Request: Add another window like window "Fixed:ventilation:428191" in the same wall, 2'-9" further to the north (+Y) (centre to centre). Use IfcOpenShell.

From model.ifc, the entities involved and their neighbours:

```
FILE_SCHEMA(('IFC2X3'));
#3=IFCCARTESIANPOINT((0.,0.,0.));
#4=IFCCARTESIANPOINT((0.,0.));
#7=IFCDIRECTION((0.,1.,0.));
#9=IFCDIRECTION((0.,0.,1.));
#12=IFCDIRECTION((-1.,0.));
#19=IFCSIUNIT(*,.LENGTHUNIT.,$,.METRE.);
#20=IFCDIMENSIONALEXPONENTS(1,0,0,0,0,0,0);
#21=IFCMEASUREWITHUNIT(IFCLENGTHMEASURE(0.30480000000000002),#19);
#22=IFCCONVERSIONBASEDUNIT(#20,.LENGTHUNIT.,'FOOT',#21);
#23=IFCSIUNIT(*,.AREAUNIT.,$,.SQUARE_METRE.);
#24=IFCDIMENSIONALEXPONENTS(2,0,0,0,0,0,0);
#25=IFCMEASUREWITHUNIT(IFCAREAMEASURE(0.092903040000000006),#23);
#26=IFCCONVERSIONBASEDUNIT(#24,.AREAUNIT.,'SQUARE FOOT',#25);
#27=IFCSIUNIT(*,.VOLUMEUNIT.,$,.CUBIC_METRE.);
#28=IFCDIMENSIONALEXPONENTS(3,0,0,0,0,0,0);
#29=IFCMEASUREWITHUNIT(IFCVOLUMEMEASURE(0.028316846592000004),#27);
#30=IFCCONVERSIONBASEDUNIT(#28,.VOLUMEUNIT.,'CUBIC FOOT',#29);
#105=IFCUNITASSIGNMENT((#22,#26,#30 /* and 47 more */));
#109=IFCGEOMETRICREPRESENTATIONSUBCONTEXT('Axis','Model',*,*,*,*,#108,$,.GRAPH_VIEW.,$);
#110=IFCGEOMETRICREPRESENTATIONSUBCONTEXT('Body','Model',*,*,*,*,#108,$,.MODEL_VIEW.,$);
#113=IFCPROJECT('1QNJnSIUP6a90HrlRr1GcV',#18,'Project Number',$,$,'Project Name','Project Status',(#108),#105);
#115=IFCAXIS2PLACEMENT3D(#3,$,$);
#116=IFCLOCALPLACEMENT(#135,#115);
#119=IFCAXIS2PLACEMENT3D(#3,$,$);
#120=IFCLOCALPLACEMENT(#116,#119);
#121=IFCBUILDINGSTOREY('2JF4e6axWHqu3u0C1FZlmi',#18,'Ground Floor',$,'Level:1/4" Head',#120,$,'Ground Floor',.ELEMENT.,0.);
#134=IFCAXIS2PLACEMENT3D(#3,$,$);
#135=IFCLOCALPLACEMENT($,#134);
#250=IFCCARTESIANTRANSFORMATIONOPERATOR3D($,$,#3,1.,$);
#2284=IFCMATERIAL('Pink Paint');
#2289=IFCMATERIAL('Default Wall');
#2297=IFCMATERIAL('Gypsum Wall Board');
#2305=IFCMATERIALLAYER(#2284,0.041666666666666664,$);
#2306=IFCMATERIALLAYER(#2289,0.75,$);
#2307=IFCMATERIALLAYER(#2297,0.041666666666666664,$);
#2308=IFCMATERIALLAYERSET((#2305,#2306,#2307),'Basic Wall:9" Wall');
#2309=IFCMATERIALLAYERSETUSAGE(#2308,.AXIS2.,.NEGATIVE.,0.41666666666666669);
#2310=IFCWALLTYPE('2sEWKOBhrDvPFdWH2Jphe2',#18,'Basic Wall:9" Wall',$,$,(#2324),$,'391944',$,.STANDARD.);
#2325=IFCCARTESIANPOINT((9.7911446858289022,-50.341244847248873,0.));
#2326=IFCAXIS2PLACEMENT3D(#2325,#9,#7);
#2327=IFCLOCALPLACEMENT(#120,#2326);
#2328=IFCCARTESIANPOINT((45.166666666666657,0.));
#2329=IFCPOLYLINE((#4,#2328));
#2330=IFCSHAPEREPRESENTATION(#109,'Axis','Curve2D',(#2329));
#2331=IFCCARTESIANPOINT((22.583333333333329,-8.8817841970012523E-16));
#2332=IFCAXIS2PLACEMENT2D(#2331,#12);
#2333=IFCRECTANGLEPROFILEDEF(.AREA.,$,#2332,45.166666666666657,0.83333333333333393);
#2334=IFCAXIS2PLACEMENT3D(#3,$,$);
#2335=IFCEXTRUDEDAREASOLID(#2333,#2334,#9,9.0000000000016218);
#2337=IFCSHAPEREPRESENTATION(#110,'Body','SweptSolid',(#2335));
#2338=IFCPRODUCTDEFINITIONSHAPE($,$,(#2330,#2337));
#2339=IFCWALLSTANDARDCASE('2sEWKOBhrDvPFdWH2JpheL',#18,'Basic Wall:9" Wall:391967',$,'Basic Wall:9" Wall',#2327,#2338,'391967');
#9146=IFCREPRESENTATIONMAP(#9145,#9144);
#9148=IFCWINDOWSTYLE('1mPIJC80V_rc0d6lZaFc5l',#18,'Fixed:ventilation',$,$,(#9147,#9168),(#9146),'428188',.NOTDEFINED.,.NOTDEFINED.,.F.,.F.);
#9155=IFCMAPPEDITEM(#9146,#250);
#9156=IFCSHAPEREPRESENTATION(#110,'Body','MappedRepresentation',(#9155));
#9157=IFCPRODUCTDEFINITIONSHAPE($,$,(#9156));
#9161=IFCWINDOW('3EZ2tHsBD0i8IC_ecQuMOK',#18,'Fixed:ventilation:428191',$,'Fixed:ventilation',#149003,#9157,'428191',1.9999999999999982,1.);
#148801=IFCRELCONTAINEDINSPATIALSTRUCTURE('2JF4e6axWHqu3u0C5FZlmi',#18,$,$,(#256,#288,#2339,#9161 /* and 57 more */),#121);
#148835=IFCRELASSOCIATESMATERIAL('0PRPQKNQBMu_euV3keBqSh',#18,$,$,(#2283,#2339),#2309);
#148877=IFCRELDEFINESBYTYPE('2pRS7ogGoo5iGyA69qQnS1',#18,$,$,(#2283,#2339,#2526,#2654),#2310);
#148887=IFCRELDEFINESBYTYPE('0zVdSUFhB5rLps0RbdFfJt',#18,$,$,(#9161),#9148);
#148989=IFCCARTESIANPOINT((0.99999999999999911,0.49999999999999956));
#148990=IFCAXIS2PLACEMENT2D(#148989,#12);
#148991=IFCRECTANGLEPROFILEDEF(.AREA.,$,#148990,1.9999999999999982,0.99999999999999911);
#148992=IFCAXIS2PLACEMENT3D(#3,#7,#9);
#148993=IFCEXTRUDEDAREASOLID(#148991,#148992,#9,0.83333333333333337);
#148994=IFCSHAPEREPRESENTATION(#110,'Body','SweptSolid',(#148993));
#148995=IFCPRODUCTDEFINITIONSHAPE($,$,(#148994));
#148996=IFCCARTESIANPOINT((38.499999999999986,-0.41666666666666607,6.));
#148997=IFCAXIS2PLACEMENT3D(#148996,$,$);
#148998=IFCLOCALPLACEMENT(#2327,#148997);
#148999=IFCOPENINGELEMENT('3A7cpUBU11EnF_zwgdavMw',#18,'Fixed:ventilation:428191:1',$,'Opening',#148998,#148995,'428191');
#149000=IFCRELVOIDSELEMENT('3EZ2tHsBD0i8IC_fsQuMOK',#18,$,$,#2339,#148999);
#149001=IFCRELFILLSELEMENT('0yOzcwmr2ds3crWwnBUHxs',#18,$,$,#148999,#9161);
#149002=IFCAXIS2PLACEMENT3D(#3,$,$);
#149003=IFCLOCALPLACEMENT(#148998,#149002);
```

```python
import ifcopenshell
import ifcopenshell.api.feature
import ifcopenshell.api.geometry
import ifcopenshell.api.root
import ifcopenshell.geom
import ifcopenshell.util.element
import ifcopenshell.util.placement
import ifcopenshell.util.shape
import ifcopenshell.util.unit

model = ifcopenshell.open("model.ifc")
unit_scale = ifcopenshell.util.unit.calculate_unit_scale(model)
settings = ifcopenshell.geom.settings()


def volume(element):
    """Net volume in cubic metres, openings subtracted."""
    shape = ifcopenshell.geom.create_shape(settings, element)
    return ifcopenshell.util.shape.get_volume(shape.geometry)


def reuse_history(source, copy):
    """copy_class also copies each property set's owner history, people and application; keep the originals."""
    for rel in copy.IsDefinedBy:
        if rel.is_a("IfcRelDefinesByProperties") and (history := rel.RelatingPropertyDefinition.OwnerHistory):
            rel.RelatingPropertyDefinition.OwnerHistory = source.OwnerHistory
            ifcopenshell.util.element.remove_deep2(model, history)


window = model.by_guid("3EZ2tHsBD0i8IC_ecQuMOK")
opening = window.FillsVoids[0].RelatingOpeningElement
wall = opening.VoidsElements[0].RelatingBuildingElement
before = volume(wall)
shift = ifcopenshell.util.placement.get_local_placement(wall.ObjectPlacement)[:3, 0] * 33 * 0.0254 / unit_scale

# copy_class copies the void relationship, type, container and properties, but no geometry.
new_opening = ifcopenshell.api.root.copy_class(model, product=opening)
new_opening.Representation = ifcopenshell.util.element.copy_deep(
    model, opening.Representation, exclude=["IfcGeometricRepresentationContext", "IfcRepresentationMap"]
)
new_opening.Name = "Fixed:ventilation"
new_opening.Tag = None
new_window = ifcopenshell.api.root.copy_class(model, product=window)
new_window.Representation = ifcopenshell.util.element.copy_deep(
    model, window.Representation, exclude=["IfcGeometricRepresentationContext", "IfcRepresentationMap"]
)
new_window.Name = "Fixed:ventilation"
new_window.Tag = None
reuse_history(window, new_window)
fills = ifcopenshell.api.feature.add_filling(model, opening=new_opening, element=new_window)
fills.OwnerHistory = new_window.OwnerHistory  # required in IFC2X3

for old, new in ((opening, new_opening), (window, new_window)):
    matrix = ifcopenshell.util.placement.get_local_placement(old.ObjectPlacement)
    matrix[:3, 3] += shift
    ifcopenshell.api.geometry.edit_object_placement(model, product=new, matrix=matrix, is_si=False)

after = volume(wall)

print(f"wall volume {before:.3f} -> {after:.3f} m3")

model.write("model-out.ifc")
```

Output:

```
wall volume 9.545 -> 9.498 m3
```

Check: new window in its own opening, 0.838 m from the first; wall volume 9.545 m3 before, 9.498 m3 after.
